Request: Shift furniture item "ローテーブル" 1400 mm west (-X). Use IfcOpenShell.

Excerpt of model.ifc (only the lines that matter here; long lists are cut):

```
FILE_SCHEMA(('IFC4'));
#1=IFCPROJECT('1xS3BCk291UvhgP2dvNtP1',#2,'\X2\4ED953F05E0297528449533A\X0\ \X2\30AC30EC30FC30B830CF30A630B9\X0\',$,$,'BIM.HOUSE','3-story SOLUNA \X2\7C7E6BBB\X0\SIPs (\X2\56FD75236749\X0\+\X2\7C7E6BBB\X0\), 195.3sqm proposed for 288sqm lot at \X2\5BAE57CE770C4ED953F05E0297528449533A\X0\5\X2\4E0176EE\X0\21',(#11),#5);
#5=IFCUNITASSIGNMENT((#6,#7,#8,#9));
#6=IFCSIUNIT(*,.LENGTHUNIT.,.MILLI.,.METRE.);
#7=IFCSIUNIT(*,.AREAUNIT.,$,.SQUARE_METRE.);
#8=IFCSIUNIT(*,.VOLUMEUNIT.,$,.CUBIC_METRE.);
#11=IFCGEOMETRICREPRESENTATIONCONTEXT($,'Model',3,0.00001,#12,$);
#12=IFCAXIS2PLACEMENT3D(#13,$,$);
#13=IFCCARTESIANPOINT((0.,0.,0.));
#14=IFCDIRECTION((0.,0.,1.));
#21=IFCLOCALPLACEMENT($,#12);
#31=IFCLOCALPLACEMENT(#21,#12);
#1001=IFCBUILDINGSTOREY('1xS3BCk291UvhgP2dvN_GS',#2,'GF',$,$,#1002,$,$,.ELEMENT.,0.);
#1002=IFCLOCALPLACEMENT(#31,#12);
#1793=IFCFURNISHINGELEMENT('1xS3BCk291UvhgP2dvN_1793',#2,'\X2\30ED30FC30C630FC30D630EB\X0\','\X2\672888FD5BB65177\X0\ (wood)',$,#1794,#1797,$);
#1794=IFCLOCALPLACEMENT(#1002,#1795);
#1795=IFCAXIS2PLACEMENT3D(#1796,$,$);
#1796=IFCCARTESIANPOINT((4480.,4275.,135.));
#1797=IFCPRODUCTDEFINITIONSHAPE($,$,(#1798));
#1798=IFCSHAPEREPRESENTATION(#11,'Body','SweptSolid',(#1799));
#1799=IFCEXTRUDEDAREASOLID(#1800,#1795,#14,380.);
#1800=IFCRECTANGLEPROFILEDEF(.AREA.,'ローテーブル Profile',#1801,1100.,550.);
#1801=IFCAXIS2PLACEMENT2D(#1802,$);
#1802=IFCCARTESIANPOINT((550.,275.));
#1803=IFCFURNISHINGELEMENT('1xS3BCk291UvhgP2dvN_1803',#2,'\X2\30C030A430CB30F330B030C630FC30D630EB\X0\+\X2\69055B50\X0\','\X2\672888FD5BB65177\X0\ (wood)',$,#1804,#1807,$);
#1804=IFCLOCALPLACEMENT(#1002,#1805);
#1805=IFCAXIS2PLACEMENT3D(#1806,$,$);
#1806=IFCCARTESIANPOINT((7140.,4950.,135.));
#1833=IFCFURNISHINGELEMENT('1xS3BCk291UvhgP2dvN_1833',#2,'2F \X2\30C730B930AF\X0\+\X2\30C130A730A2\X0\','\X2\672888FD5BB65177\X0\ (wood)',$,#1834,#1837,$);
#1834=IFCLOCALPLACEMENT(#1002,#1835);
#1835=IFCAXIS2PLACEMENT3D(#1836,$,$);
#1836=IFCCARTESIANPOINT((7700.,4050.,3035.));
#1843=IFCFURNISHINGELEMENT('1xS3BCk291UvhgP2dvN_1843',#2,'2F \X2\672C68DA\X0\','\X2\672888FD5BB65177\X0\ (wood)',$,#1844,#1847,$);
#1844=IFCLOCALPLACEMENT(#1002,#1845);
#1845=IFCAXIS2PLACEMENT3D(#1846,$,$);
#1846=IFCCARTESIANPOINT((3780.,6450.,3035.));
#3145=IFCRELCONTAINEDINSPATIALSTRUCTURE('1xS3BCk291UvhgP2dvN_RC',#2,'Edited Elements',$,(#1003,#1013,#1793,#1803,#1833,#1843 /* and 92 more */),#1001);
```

```python
import ifcopenshell
import ifcopenshell.api.geometry
import ifcopenshell.util.placement

model = ifcopenshell.open("model.ifc")

item = model.by_guid("1xS3BCk291UvhgP2dvN_1793")
matrix = ifcopenshell.util.placement.get_local_placement(item.ObjectPlacement)
matrix[0, 3] -= 1400.0
ifcopenshell.api.geometry.edit_object_placement(model, product=item, matrix=matrix, is_si=False)

print(ifcopenshell.util.placement.get_local_placement(item.ObjectPlacement).round(3) + 0.0)

model.write("model_updated.ifc")
```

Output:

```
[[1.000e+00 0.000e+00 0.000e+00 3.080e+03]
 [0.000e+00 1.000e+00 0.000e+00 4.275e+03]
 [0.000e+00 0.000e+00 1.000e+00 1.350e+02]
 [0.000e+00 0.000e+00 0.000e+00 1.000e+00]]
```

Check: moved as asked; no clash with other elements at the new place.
